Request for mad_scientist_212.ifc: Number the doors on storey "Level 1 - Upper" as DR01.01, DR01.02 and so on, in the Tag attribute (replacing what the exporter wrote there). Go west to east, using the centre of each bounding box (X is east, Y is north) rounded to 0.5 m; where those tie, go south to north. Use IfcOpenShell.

First a look at what the model holds.

```python
import ifcopenshell
import ifcopenshell.util.element
import ifcopenshell.util.placement

model = ifcopenshell.open("mad_scientist_212.ifc")
print(model.schema)
storey = next(s for s in model.by_type("IfcBuildingStorey") if s.Name == "Level 1 - Upper")
doors = [e for e in ifcopenshell.util.element.get_decomposition(storey) if e.is_a("IfcDoor")]
for e in sorted(doors, key=lambda e: e.id()):
    origin = ifcopenshell.util.placement.get_local_placement(e.ObjectPlacement)[:3, 3]
    print(e.id(), e.Tag, e.Name, origin.round(2) + 0.0, sep=" | ")
```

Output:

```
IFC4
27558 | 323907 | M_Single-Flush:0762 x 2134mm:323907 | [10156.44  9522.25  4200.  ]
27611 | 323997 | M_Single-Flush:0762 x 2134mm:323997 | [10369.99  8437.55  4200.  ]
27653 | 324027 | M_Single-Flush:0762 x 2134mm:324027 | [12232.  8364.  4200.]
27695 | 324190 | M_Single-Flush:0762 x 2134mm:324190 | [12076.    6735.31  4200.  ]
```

```python
import ifcopenshell
import ifcopenshell.geom
import ifcopenshell.util.element
import ifcopenshell.util.shape

model = ifcopenshell.open("mad_scientist_212.ifc")
settings = ifcopenshell.geom.settings()
settings.set("use-world-coords", True)


def centre(element):
    shape = ifcopenshell.geom.create_shape(settings, element)
    return ifcopenshell.util.shape.get_bbox_centroid(shape.geometry)


storey = next(s for s in model.by_type("IfcBuildingStorey") if s.Name == "Level 1 - Upper")
doors = [e for e in ifcopenshell.util.element.get_decomposition(storey) if e.is_a("IfcDoor")]

# Insertion points can sit at a corner or the storey origin, so sort by the geometry (in metres).
centres = {e: centre(e) for e in doors}
doors.sort(key=lambda e: (round(centres[e][0] / 0.5), centres[e][1]))

for i, e in enumerate(doors, start=1):
    number = f"DR01.{i:02d}"
    e.Tag = number
    print(e.id(), number)

model.write("mad_scientist_212-out.ifc")
```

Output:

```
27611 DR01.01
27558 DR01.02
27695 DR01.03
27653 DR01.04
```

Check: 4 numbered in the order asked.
